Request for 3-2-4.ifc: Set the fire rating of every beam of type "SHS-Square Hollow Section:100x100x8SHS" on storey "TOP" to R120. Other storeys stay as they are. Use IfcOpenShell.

First a look at what the model holds.

```python
import ifcopenshell
import ifcopenshell.util.element

model = ifcopenshell.open("3-2-4.ifc")
print(model.schema)
storey = next(s for s in model.by_type("IfcBuildingStorey") if s.Name == "TOP")
beams = [e for e in ifcopenshell.util.element.get_decomposition(storey) if e.is_a("IfcBeam")]
seen = {}
for e in beams:
    element_type = ifcopenshell.util.element.get_type(e)
    key = (element_type.Name if element_type != e and element_type else None, ifcopenshell.util.element.get_pset(e, "Pset_BeamCommon", "FireRating"))
    seen[key] = seen.get(key, 0) + 1
for (name, value), count in sorted(seen.items(), key=str):
    print(count, "x", name, "|", value)
```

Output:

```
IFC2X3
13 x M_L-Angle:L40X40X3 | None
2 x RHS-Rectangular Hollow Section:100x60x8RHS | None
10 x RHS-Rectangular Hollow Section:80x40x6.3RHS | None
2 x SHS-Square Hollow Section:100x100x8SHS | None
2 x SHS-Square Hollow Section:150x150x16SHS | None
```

```python
import ifcopenshell
import ifcopenshell.api.pset
import ifcopenshell.util.element

model = ifcopenshell.open("3-2-4.ifc")

storey = next(s for s in model.by_type("IfcBuildingStorey") if s.Name == "TOP")
beams = [e for e in ifcopenshell.util.element.get_decomposition(storey) if e.is_a("IfcBeam")]

count = 0
for e in beams:
    element_type = ifcopenshell.util.element.get_type(e)
    if element_type in (None, e) or element_type.Name != "SHS-Square Hollow Section:100x100x8SHS":
        continue
    # add_pset returns the element's existing set when there is one.
    pset = ifcopenshell.api.pset.add_pset(model, product=e, name="Pset_BeamCommon")
    ifcopenshell.api.pset.edit_pset(model, pset=pset, properties={"FireRating": "R120"})
    count += 1

print(count, "beams updated")

model.write("3-2-4_updated.ifc")
```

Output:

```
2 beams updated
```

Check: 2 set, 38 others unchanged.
